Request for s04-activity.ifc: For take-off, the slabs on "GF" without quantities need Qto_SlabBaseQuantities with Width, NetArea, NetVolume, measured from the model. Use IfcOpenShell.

First a look at what the model holds.

```python
import ifcopenshell
import ifcopenshell.util.element
import ifcopenshell.util.unit

model = ifcopenshell.open("s04-activity.ifc")
print(model.schema)
for unit_type in ("LENGTHUNIT", "AREAUNIT", "VOLUMEUNIT"):
    print(unit_type, ifcopenshell.util.unit.calculate_unit_scale(model, unit_type))
storey = next(s for s in model.by_type("IfcBuildingStorey") if s.Name == "GF")
slabs = [e for e in ifcopenshell.util.element.get_decomposition(storey) if e.is_a("IfcSlab")]
for e in sorted(slabs, key=lambda e: e.id()):
    print(e.id(), e.is_a(), e.Name, list(ifcopenshell.util.element.get_psets(e, qtos_only=True)), sep=" | ")
```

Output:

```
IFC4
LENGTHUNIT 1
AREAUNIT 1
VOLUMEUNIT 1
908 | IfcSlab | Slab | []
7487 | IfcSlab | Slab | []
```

```python
import ifcopenshell
import ifcopenshell.api.pset
import ifcopenshell.geom
import ifcopenshell.util.element
import ifcopenshell.util.shape
import ifcopenshell.util.unit

model = ifcopenshell.open("s04-activity.ifc")
unit_scale = ifcopenshell.util.unit.calculate_unit_scale(model)
area_scale = ifcopenshell.util.unit.calculate_unit_scale(model, "AREAUNIT")
volume_scale = ifcopenshell.util.unit.calculate_unit_scale(model, "VOLUMEUNIT")
settings = ifcopenshell.geom.settings()

storey = next(s for s in model.by_type("IfcBuildingStorey") if s.Name == "GF")
slabs = [e for e in ifcopenshell.util.element.get_decomposition(storey) if e.is_a("IfcSlab")]

for e in sorted(slabs, key=lambda e: e.id()):
    if ifcopenshell.util.element.get_psets(e, qtos_only=True, should_inherit=False):
        continue
    # Geometry comes back in metres, in the element's own axes.
    shape = ifcopenshell.geom.create_shape(settings, e)
    values = {
        "Width": ifcopenshell.util.shape.get_z(shape.geometry) / unit_scale,
        "NetArea": ifcopenshell.util.shape.get_footprint_area(shape.geometry) / area_scale,
        "NetVolume": ifcopenshell.util.shape.get_volume(shape.geometry) / volume_scale,
    }
    qto = ifcopenshell.api.pset.add_qto(model, product=e, name="Qto_SlabBaseQuantities")
    ifcopenshell.api.pset.edit_qto(model, qto=qto, properties=values)
    print(e.id(), {k: round(v, 3) for k, v in values.items()})

model.write("s04-activity_updated.ifc")
```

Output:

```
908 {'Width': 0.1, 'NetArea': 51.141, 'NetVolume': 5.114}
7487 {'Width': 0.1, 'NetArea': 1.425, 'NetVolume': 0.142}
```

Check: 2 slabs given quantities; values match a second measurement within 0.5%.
